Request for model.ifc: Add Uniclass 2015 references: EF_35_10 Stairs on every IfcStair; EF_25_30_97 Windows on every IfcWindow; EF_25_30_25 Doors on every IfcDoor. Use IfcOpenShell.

First a look at what the model holds.

```python
import ifcopenshell

model = ifcopenshell.open("model.ifc")
print(model.schema)
print("classifications:", [c.Name for c in model.by_type("IfcClassification")])
for ifc_class in ("IfcDoor", "IfcRoof", "IfcStair", "IfcWall", "IfcWindow"):
    print(ifc_class, len(model.by_type(ifc_class)))
```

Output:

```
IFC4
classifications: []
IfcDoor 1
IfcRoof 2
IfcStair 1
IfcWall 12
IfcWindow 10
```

```python
import ifcopenshell
import ifcopenshell.api.classification

model = ifcopenshell.open("model.ifc")

system = ifcopenshell.api.classification.add_classification(model, classification="Uniclass 2015")

codes = {
    "IfcStair": ("EF_35_10", "Stairs"),
    "IfcWindow": ("EF_25_30_97", "Windows"),
    "IfcDoor": ("EF_25_30_25", "Doors"),
}
for ifc_class, (code, name) in codes.items():
    products = model.by_type(ifc_class)
    ifcopenshell.api.classification.add_reference(
        model, products=products, classification=system, identification=code, name=name
    )
    print(code, len(products))

model.write("model_updated.ifc")
```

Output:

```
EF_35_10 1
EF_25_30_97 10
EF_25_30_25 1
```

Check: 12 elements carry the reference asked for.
